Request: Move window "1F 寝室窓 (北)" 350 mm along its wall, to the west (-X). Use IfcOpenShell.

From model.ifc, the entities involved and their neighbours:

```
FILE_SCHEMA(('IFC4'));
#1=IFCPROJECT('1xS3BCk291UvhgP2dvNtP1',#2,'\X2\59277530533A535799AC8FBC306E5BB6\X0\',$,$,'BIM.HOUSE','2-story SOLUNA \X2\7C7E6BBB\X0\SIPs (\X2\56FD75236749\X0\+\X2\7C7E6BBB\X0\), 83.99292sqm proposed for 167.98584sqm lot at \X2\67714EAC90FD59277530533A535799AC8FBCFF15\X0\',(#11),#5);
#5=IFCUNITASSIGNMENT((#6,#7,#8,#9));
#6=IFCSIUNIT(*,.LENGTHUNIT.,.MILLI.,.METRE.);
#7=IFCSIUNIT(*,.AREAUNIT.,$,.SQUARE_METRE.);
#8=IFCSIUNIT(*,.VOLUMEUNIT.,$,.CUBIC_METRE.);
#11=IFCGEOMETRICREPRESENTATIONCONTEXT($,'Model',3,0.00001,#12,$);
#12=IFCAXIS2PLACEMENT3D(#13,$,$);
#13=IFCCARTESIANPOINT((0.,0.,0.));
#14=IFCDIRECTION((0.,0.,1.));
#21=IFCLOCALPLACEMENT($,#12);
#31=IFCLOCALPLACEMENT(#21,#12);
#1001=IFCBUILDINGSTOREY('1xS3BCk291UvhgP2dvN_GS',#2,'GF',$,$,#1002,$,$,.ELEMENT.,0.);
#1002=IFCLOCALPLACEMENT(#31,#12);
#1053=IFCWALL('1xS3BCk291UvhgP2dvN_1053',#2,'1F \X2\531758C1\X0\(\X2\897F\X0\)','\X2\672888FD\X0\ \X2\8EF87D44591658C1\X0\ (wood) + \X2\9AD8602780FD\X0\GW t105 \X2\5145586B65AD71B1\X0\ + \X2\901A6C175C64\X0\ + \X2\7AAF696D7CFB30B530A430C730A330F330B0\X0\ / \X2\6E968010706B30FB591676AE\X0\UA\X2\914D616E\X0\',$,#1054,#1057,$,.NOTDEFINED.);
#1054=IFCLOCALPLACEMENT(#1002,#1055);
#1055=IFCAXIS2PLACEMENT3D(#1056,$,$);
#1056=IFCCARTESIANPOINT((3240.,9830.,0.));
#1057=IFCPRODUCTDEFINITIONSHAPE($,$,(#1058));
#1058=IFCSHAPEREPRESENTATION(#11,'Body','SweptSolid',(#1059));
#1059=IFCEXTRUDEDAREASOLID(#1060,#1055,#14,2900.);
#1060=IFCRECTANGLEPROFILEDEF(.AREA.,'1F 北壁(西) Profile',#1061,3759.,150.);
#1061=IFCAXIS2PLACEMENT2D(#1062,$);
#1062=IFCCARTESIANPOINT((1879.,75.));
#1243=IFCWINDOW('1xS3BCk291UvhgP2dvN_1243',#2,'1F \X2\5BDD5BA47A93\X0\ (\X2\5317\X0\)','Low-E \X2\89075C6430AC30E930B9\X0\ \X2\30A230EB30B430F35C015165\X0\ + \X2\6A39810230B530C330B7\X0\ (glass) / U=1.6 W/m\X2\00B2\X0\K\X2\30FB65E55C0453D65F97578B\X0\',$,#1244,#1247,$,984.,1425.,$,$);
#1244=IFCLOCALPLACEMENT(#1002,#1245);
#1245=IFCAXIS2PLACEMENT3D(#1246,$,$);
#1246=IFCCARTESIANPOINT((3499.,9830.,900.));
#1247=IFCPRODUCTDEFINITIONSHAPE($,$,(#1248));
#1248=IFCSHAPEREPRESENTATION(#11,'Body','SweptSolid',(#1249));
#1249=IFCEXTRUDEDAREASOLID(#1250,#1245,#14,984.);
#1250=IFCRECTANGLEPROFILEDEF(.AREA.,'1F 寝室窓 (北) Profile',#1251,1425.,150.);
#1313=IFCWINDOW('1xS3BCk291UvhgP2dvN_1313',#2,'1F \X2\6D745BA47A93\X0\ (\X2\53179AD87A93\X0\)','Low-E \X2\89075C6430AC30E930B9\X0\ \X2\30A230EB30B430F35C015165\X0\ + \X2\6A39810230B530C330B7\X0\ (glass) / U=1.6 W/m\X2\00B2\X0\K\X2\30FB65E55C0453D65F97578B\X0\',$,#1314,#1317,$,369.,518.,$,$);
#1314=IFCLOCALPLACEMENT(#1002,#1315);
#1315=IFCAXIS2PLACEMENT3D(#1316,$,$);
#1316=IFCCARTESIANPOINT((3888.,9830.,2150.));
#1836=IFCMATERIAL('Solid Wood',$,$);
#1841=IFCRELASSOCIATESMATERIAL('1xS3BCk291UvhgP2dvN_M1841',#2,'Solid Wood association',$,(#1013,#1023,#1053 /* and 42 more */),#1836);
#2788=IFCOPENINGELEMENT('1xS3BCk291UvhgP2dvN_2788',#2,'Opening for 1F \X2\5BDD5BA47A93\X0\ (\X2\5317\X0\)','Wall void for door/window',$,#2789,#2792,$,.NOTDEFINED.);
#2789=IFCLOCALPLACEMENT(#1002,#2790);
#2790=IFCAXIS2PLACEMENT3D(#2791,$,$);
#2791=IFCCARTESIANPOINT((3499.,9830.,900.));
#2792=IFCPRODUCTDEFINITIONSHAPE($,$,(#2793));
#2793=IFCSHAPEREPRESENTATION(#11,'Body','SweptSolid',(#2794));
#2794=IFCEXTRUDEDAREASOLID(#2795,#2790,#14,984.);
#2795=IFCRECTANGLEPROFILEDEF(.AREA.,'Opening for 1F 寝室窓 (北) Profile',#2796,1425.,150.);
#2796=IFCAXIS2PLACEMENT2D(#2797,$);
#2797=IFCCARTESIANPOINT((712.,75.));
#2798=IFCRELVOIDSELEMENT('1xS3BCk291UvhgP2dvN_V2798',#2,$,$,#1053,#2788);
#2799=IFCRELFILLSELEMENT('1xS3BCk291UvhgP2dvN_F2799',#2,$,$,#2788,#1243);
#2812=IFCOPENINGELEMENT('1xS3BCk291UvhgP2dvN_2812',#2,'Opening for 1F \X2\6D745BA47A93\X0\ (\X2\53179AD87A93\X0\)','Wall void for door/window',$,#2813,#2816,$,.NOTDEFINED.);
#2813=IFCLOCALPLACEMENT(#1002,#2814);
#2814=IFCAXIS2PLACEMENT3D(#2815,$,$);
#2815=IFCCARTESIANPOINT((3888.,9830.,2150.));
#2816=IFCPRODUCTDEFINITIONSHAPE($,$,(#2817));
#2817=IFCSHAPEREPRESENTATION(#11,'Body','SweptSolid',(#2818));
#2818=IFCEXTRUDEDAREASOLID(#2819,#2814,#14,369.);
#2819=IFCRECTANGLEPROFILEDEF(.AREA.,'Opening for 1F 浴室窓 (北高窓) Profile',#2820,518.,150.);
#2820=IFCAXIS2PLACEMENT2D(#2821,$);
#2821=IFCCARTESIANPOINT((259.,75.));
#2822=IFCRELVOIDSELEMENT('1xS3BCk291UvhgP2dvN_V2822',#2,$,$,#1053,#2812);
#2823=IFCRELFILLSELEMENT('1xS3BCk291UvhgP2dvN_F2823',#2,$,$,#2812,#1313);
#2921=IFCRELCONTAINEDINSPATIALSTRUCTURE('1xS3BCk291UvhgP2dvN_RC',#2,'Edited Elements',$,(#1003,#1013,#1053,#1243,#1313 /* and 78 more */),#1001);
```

```python
import ifcopenshell
import ifcopenshell.api.geometry
import ifcopenshell.util.placement

model = ifcopenshell.open("model.ifc")

window = model.by_guid("1xS3BCk291UvhgP2dvN_1243")
opening = window.FillsVoids[0].RelatingOpeningElement
wall = opening.VoidsElements[0].RelatingBuildingElement

wall_matrix = ifcopenshell.util.placement.get_local_placement(wall.ObjectPlacement)
shift = wall_matrix[:3, 0] * -350.0
before = ifcopenshell.util.placement.get_local_placement(window.ObjectPlacement)[:3, 3].copy()

# The window is not placed relative to its opening, so move both.
for product in (opening, window):
    matrix = ifcopenshell.util.placement.get_local_placement(product.ObjectPlacement)
    matrix[:3, 3] += shift
    ifcopenshell.api.geometry.edit_object_placement(model, product=product, matrix=matrix, is_si=False)

after = ifcopenshell.util.placement.get_local_placement(window.ObjectPlacement)[:3, 3]
print("window moved by", (after - before).round(3) + 0.0)

model.write("model-out.ifc")
```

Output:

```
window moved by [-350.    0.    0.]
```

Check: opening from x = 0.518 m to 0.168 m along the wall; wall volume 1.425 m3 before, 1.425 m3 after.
